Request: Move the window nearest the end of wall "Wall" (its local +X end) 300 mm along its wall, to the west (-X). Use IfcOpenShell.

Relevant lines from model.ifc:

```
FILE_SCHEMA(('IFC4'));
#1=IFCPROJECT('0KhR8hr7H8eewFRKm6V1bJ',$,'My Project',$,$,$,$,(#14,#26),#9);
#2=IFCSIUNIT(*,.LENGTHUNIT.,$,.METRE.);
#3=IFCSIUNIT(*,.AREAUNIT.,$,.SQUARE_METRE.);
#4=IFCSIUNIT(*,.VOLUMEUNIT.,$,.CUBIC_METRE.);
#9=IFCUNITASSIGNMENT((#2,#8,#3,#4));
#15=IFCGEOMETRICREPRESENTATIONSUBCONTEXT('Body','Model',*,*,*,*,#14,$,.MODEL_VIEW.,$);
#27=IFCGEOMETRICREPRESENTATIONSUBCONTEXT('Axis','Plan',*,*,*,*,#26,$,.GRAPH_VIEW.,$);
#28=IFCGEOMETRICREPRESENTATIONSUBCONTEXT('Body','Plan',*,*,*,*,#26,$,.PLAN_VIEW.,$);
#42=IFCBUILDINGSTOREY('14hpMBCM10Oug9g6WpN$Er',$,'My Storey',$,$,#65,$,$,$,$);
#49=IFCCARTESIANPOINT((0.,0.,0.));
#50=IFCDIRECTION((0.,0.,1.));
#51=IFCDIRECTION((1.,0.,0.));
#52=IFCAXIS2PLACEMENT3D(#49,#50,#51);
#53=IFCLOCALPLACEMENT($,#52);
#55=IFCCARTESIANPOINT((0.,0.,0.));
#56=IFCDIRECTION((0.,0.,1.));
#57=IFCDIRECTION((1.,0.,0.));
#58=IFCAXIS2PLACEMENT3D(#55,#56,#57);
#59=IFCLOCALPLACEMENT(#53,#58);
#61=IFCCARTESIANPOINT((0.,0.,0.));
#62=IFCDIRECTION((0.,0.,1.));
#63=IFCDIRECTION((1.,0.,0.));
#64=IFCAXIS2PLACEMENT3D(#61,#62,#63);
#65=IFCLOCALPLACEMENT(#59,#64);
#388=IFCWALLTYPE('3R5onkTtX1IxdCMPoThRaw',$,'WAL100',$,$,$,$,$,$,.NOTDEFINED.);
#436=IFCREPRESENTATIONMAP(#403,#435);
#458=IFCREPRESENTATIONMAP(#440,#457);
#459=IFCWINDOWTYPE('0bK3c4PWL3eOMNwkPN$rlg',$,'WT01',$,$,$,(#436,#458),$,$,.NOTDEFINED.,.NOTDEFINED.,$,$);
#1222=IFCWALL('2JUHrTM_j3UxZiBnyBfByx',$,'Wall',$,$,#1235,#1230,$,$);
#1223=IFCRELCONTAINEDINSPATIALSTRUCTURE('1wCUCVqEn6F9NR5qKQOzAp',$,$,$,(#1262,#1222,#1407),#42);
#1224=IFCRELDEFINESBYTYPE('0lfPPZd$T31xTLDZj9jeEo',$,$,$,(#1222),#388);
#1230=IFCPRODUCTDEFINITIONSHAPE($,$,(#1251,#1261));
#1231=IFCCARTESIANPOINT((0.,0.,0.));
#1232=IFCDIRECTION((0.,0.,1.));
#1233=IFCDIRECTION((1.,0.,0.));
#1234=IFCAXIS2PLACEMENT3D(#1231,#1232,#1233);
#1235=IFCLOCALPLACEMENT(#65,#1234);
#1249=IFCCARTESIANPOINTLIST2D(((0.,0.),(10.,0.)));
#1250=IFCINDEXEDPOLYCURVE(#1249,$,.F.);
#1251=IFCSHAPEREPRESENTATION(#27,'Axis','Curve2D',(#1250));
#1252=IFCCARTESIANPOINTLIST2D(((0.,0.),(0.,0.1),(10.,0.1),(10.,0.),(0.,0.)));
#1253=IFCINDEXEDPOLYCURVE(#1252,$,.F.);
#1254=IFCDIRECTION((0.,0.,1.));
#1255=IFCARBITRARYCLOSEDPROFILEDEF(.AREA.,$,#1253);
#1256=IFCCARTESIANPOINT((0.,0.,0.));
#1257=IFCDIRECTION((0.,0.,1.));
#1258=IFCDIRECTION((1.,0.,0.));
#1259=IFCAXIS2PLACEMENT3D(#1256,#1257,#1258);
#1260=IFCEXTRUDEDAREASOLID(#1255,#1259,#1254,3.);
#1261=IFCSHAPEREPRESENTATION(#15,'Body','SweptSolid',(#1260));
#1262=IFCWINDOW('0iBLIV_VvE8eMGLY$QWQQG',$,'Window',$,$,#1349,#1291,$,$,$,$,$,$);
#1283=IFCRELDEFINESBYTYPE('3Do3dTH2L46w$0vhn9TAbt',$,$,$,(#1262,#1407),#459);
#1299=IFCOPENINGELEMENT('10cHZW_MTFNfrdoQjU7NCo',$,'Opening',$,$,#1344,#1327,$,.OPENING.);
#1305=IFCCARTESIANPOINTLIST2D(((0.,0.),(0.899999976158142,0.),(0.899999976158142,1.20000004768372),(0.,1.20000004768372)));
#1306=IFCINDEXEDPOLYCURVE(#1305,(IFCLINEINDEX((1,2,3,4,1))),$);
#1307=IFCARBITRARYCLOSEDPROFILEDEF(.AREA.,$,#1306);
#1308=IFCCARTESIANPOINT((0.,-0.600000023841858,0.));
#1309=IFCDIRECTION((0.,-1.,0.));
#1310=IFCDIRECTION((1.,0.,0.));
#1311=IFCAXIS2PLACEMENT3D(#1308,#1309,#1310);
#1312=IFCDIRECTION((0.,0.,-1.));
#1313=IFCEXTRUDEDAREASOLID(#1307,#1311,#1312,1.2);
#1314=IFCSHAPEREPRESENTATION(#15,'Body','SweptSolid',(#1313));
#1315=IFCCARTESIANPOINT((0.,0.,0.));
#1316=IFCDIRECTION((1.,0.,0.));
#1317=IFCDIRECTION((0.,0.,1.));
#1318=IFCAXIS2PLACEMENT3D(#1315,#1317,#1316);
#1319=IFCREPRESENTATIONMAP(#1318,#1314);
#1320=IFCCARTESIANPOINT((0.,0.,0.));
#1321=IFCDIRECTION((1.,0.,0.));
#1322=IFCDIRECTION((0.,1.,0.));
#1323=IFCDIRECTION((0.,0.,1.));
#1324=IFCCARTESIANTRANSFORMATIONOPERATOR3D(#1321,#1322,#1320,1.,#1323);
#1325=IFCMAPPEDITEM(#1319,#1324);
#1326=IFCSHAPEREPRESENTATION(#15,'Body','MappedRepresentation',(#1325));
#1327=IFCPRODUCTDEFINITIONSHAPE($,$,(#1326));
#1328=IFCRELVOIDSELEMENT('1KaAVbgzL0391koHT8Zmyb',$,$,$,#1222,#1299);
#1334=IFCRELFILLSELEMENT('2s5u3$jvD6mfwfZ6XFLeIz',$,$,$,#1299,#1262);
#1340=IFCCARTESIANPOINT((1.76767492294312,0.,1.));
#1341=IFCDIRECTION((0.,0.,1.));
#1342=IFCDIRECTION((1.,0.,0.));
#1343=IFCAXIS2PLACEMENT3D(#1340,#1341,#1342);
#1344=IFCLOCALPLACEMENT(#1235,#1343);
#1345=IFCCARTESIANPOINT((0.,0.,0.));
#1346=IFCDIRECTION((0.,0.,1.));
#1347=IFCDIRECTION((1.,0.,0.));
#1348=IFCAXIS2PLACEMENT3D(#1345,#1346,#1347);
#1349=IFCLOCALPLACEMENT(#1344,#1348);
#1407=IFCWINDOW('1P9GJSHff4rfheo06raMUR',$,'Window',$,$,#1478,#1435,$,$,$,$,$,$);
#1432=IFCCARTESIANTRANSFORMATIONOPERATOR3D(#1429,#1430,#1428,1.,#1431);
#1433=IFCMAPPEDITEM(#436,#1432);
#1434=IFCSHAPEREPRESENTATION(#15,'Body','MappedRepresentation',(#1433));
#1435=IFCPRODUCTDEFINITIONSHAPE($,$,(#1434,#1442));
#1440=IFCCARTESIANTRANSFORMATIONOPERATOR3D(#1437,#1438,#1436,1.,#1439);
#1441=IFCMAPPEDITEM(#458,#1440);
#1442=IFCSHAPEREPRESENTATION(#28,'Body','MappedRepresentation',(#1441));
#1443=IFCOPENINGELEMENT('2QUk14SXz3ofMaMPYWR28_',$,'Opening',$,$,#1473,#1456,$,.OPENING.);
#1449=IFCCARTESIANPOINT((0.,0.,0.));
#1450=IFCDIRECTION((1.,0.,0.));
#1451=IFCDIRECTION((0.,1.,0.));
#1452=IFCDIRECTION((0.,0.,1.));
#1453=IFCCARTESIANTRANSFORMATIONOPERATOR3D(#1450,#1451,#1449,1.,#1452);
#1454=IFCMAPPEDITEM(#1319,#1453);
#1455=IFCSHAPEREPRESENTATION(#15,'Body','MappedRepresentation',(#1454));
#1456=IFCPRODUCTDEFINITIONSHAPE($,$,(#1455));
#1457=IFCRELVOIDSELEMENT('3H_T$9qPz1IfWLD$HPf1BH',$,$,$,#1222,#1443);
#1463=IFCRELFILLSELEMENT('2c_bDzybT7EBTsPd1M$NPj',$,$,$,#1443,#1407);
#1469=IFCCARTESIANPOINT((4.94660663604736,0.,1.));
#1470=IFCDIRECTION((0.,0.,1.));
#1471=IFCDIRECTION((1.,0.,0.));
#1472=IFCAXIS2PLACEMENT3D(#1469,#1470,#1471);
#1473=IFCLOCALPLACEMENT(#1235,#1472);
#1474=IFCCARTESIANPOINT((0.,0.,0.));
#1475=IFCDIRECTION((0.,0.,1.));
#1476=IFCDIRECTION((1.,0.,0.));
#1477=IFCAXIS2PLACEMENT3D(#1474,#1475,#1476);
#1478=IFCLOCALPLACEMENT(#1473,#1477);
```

```python
import ifcopenshell
import ifcopenshell.api.geometry
import ifcopenshell.util.placement

model = ifcopenshell.open("model.ifc")

window = model.by_guid("1P9GJSHff4rfheo06raMUR")
opening = window.FillsVoids[0].RelatingOpeningElement
wall = opening.VoidsElements[0].RelatingBuildingElement

wall_matrix = ifcopenshell.util.placement.get_local_placement(wall.ObjectPlacement)
shift = wall_matrix[:3, 0] * -0.3
before = ifcopenshell.util.placement.get_local_placement(window.ObjectPlacement)[:3, 3].copy()

# The window is placed relative to its opening, so it follows when the opening moves.
matrix = ifcopenshell.util.placement.get_local_placement(opening.ObjectPlacement)
matrix[:3, 3] += shift
ifcopenshell.api.geometry.edit_object_placement(
    model, product=opening, matrix=matrix, is_si=False, should_transform_children=True
)

after = ifcopenshell.util.placement.get_local_placement(window.ObjectPlacement)[:3, 3]
print("window moved by", (after - before).round(3) + 0.0)

model.write("model_updated.ifc")
```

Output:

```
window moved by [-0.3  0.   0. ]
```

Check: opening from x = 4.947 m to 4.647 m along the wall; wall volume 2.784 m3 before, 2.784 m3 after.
